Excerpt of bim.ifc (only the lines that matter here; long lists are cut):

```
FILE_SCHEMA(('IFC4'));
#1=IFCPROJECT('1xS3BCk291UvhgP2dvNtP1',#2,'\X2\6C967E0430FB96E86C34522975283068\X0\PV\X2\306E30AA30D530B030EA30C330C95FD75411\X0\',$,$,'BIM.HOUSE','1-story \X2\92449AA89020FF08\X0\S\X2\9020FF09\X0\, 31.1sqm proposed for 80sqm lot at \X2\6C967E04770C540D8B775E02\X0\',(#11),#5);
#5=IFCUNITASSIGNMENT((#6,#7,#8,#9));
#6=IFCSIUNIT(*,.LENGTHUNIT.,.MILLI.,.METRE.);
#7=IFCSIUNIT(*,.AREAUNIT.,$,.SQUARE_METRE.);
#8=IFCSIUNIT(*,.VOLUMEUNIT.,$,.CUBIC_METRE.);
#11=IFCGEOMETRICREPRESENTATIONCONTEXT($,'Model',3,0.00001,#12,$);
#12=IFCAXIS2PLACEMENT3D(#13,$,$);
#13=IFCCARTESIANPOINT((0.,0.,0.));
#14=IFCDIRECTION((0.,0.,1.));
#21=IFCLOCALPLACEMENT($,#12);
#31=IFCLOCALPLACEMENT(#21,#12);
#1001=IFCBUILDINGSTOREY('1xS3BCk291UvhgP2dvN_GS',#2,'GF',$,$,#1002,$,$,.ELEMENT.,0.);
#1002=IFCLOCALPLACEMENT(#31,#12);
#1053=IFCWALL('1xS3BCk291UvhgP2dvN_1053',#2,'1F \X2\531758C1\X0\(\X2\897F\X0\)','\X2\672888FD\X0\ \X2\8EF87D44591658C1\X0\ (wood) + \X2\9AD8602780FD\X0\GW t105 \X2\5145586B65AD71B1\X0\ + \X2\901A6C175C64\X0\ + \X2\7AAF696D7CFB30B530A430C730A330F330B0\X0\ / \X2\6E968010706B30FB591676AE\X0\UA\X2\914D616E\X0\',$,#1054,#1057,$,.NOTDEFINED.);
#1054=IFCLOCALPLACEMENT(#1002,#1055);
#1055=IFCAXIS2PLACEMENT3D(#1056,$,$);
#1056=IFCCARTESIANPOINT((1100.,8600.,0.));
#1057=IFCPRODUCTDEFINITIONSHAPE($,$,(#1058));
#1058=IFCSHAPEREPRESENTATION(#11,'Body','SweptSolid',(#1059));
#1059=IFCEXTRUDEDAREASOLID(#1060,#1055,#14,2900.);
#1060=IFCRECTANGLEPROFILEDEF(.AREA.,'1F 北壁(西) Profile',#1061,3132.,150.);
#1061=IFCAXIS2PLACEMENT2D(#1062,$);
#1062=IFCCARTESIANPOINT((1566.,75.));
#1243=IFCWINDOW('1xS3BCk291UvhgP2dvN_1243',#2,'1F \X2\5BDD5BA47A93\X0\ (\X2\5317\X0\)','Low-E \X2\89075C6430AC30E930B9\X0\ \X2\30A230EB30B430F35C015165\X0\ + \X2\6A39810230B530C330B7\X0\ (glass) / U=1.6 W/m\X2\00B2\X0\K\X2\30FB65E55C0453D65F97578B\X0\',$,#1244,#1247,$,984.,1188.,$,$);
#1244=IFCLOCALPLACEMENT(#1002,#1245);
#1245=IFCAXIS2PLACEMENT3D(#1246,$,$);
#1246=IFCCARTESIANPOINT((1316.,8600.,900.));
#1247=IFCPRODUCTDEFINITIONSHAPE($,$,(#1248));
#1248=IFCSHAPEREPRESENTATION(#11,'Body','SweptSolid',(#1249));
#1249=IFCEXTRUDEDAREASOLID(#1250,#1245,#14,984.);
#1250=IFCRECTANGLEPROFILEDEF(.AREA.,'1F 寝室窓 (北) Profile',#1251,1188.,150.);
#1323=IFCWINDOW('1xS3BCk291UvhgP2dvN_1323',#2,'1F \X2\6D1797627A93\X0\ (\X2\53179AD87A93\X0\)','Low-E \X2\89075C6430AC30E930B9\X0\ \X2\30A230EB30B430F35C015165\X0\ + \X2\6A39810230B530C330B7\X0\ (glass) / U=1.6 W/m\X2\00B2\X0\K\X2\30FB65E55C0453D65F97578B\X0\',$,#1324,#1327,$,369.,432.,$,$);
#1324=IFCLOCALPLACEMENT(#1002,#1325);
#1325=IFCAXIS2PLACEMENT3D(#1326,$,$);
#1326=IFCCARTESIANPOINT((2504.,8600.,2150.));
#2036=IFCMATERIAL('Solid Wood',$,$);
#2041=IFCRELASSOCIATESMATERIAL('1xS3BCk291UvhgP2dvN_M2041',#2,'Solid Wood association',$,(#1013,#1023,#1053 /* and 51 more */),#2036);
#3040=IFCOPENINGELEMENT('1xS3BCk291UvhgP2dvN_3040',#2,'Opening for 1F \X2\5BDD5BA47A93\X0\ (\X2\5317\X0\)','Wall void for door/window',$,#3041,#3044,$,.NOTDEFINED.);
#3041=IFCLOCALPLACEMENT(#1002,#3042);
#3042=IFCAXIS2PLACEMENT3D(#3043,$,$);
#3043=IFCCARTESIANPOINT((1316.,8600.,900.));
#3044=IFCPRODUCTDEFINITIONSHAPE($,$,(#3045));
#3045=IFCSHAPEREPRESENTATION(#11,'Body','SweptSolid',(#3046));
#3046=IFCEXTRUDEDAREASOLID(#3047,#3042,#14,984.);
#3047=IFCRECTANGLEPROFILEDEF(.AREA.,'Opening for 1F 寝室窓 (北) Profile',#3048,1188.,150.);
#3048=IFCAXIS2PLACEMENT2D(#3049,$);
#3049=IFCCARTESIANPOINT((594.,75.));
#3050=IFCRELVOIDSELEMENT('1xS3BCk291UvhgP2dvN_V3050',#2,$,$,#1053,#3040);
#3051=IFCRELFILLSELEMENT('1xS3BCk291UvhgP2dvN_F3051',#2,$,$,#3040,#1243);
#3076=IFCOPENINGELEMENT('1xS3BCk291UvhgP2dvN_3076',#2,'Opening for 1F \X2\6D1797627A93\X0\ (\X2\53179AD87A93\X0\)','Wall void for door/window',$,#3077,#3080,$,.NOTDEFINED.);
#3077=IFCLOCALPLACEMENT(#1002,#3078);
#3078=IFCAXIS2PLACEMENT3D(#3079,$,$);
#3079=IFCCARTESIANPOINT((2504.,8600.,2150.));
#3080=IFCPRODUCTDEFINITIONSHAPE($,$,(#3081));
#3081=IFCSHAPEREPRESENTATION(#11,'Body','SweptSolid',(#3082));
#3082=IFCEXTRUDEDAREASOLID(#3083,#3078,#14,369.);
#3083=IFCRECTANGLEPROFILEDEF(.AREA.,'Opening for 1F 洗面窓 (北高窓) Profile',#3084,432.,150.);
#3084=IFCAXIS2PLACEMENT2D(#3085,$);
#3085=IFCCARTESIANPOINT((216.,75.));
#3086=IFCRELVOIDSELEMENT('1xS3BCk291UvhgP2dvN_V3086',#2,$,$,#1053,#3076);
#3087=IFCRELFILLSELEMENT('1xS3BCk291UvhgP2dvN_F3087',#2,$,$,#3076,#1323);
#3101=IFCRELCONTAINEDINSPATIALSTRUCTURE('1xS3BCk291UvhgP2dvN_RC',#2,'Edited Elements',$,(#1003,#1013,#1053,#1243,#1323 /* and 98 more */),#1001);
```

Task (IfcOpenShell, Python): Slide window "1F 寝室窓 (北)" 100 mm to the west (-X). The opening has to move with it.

```python
import ifcopenshell
import ifcopenshell.api.geometry
import ifcopenshell.util.placement
import ifcopenshell.util.unit

model = ifcopenshell.open("bim.ifc")
unit_scale = ifcopenshell.util.unit.calculate_unit_scale(model)

window = model.by_guid("1xS3BCk291UvhgP2dvN_1243")
opening = window.FillsVoids[0].RelatingOpeningElement
wall = opening.VoidsElements[0].RelatingBuildingElement

wall_matrix = ifcopenshell.util.placement.get_local_placement(wall.ObjectPlacement)
shift = wall_matrix[:3, 0] * -0.1 / unit_scale
before = ifcopenshell.util.placement.get_local_placement(window.ObjectPlacement)[:3, 3].copy()

# The window is not placed relative to its opening, so move both.
for product in (opening, window):
    matrix = ifcopenshell.util.placement.get_local_placement(product.ObjectPlacement)
    matrix[:3, 3] += shift
    ifcopenshell.api.geometry.edit_object_placement(model, product=product, matrix=matrix, is_si=False)

after = ifcopenshell.util.placement.get_local_placement(window.ObjectPlacement)[:3, 3]
print("window moved by", (after - before).round(3) + 0.0)

model.write("bim-out.ifc")
```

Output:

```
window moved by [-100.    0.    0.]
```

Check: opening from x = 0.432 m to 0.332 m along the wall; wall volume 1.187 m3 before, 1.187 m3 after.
